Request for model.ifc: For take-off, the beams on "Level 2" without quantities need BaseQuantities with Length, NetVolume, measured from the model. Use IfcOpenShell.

First a look at what the model holds.

```python
import ifcopenshell
import ifcopenshell.util.element
import ifcopenshell.util.unit

model = ifcopenshell.open("model.ifc")
print(model.schema)
for unit_type in ("LENGTHUNIT", "AREAUNIT", "VOLUMEUNIT"):
    print(unit_type, ifcopenshell.util.unit.calculate_unit_scale(model, unit_type))
storey = next(s for s in model.by_type("IfcBuildingStorey") if s.Name == "Level 2")
beams = [e for e in ifcopenshell.util.element.get_decomposition(storey) if e.is_a("IfcBeam")]
for e in sorted(beams, key=lambda e: e.id()):
    print(e.id(), e.is_a(), e.Name, list(ifcopenshell.util.element.get_psets(e, qtos_only=True)), sep=" | ")
```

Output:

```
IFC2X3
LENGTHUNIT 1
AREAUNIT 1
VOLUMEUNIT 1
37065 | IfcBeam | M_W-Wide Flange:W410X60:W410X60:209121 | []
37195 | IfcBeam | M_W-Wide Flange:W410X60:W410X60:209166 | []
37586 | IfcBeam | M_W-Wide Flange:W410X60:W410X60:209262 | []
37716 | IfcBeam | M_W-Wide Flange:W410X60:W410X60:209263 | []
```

```python
import ifcopenshell
import ifcopenshell.api.pset
import ifcopenshell.geom
import ifcopenshell.util.element
import ifcopenshell.util.shape
import ifcopenshell.util.unit

model = ifcopenshell.open("model.ifc")
unit_scale = ifcopenshell.util.unit.calculate_unit_scale(model)
volume_scale = ifcopenshell.util.unit.calculate_unit_scale(model, "VOLUMEUNIT")
settings = ifcopenshell.geom.settings()

storey = next(s for s in model.by_type("IfcBuildingStorey") if s.Name == "Level 2")
beams = [e for e in ifcopenshell.util.element.get_decomposition(storey) if e.is_a("IfcBeam")]

for e in sorted(beams, key=lambda e: e.id()):
    if ifcopenshell.util.element.get_psets(e, qtos_only=True, should_inherit=False):
        continue
    # Geometry comes back in metres, in the element's own axes.
    shape = ifcopenshell.geom.create_shape(settings, e)
    values = {
        "Length": ifcopenshell.util.shape.get_max_xyz(shape.geometry) / unit_scale,
        "NetVolume": ifcopenshell.util.shape.get_volume(shape.geometry) / volume_scale,
    }
    qto = ifcopenshell.api.pset.add_qto(model, product=e, name="BaseQuantities")
    ifcopenshell.api.pset.edit_qto(model, qto=qto, properties=values)
    print(e.id(), {k: round(v, 3) for k, v in values.items()})

model.write("model_v2.ifc")
```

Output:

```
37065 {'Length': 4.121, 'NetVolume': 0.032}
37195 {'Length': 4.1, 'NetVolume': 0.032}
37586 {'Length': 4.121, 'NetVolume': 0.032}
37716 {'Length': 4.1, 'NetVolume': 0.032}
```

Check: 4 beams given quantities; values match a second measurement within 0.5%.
